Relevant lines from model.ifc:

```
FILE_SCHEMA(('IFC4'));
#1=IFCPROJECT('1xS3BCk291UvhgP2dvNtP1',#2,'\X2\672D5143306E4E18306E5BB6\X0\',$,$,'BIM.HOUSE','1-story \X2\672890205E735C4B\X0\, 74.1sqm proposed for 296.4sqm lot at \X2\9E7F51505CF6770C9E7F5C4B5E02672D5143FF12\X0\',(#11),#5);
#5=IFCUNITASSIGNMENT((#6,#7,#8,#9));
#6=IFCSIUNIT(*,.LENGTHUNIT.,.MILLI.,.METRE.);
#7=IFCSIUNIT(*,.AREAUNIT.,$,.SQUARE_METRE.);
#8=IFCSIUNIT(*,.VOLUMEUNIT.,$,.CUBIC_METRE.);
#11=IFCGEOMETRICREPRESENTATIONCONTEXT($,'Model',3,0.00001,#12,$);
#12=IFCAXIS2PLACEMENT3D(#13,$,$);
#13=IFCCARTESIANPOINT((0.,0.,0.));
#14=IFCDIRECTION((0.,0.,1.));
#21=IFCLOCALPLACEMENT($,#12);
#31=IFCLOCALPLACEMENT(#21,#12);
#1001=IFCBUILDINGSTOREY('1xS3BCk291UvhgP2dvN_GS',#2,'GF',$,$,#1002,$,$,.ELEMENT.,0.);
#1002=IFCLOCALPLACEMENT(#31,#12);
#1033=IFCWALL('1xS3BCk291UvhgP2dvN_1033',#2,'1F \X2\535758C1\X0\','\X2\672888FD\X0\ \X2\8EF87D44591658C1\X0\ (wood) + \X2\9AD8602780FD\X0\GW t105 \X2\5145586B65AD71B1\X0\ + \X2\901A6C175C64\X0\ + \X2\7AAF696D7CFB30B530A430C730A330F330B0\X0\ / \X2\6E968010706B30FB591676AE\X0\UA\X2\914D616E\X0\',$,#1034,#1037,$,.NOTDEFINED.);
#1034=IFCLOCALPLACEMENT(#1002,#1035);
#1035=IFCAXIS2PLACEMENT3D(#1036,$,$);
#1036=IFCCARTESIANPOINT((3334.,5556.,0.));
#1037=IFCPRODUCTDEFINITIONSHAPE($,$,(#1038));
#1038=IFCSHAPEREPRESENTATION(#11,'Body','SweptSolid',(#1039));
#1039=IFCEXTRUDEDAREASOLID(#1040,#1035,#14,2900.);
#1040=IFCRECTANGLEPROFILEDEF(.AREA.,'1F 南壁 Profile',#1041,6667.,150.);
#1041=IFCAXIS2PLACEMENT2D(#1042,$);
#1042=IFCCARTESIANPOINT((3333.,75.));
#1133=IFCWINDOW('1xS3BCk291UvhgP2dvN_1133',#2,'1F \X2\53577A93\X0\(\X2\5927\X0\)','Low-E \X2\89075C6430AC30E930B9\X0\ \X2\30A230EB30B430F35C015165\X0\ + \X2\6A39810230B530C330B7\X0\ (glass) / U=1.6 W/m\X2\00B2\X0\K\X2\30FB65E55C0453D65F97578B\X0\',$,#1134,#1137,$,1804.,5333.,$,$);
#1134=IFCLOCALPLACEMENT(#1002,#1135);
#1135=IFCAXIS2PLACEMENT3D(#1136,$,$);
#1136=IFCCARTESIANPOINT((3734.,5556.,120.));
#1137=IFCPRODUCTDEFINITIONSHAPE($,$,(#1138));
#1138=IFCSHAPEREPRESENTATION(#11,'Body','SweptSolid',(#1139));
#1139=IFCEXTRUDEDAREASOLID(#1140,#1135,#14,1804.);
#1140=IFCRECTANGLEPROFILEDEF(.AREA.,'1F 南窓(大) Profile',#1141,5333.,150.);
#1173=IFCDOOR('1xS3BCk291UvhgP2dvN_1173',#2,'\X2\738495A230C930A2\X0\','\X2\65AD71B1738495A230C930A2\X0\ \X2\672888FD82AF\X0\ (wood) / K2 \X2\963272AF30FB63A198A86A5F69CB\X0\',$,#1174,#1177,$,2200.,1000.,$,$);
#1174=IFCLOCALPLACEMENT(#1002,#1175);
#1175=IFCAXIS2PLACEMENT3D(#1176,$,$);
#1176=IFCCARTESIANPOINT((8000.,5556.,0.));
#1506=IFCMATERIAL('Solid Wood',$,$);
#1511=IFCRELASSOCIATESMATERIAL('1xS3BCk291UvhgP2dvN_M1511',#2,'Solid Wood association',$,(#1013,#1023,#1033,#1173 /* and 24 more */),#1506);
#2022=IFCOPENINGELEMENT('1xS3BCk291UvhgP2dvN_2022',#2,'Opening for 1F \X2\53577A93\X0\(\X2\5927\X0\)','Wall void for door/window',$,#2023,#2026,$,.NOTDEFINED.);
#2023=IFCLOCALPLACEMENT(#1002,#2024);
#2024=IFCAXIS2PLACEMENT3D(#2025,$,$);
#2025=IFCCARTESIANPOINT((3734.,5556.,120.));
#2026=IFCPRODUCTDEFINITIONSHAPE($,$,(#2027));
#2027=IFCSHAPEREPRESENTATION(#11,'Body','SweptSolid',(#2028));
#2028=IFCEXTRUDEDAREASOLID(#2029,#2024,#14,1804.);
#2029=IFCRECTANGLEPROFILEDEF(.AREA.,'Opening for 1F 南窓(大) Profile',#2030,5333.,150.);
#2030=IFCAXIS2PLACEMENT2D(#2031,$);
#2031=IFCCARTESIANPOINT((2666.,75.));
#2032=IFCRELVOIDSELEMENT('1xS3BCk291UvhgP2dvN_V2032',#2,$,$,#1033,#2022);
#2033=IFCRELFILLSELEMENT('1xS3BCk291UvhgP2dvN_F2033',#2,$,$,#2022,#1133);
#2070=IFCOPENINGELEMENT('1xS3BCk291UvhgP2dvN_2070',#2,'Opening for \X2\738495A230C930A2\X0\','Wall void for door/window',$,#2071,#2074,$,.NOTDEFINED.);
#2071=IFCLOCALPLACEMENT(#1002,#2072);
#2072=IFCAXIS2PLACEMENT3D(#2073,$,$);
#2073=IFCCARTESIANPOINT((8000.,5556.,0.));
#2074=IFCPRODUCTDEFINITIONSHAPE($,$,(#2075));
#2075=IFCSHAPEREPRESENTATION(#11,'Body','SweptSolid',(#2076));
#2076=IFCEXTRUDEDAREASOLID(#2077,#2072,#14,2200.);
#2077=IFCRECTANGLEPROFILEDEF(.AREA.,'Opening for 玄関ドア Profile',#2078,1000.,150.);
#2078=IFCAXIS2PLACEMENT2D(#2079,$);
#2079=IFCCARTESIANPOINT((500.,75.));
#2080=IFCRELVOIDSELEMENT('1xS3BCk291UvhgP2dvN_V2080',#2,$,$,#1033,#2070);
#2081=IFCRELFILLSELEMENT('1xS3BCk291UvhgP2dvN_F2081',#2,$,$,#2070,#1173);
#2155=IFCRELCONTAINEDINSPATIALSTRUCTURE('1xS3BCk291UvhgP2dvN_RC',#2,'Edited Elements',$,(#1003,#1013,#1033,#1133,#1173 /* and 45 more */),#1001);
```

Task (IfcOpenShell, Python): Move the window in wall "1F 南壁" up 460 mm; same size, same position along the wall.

```python
import numpy as np
import ifcopenshell
import ifcopenshell.api.geometry
import ifcopenshell.util.placement
import ifcopenshell.util.unit

model = ifcopenshell.open("model.ifc")
unit_scale = ifcopenshell.util.unit.calculate_unit_scale(model)

window = model.by_guid("1xS3BCk291UvhgP2dvN_1133")
opening = window.FillsVoids[0].RelatingOpeningElement
dz = 0.46 / unit_scale

shift = np.array([0.0, 0.0, dz])
# The window is not placed relative to its opening, so move both.
for product in (opening, window):
    matrix = ifcopenshell.util.placement.get_local_placement(product.ObjectPlacement)
    matrix[:3, 3] += shift
    ifcopenshell.api.geometry.edit_object_placement(model, product=product, matrix=matrix, is_si=False)

print(f"moved by {dz * unit_scale:+.3f} m")

model.write("model_edited.ifc")
```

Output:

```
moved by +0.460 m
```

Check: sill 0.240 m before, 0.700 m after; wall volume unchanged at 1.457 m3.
